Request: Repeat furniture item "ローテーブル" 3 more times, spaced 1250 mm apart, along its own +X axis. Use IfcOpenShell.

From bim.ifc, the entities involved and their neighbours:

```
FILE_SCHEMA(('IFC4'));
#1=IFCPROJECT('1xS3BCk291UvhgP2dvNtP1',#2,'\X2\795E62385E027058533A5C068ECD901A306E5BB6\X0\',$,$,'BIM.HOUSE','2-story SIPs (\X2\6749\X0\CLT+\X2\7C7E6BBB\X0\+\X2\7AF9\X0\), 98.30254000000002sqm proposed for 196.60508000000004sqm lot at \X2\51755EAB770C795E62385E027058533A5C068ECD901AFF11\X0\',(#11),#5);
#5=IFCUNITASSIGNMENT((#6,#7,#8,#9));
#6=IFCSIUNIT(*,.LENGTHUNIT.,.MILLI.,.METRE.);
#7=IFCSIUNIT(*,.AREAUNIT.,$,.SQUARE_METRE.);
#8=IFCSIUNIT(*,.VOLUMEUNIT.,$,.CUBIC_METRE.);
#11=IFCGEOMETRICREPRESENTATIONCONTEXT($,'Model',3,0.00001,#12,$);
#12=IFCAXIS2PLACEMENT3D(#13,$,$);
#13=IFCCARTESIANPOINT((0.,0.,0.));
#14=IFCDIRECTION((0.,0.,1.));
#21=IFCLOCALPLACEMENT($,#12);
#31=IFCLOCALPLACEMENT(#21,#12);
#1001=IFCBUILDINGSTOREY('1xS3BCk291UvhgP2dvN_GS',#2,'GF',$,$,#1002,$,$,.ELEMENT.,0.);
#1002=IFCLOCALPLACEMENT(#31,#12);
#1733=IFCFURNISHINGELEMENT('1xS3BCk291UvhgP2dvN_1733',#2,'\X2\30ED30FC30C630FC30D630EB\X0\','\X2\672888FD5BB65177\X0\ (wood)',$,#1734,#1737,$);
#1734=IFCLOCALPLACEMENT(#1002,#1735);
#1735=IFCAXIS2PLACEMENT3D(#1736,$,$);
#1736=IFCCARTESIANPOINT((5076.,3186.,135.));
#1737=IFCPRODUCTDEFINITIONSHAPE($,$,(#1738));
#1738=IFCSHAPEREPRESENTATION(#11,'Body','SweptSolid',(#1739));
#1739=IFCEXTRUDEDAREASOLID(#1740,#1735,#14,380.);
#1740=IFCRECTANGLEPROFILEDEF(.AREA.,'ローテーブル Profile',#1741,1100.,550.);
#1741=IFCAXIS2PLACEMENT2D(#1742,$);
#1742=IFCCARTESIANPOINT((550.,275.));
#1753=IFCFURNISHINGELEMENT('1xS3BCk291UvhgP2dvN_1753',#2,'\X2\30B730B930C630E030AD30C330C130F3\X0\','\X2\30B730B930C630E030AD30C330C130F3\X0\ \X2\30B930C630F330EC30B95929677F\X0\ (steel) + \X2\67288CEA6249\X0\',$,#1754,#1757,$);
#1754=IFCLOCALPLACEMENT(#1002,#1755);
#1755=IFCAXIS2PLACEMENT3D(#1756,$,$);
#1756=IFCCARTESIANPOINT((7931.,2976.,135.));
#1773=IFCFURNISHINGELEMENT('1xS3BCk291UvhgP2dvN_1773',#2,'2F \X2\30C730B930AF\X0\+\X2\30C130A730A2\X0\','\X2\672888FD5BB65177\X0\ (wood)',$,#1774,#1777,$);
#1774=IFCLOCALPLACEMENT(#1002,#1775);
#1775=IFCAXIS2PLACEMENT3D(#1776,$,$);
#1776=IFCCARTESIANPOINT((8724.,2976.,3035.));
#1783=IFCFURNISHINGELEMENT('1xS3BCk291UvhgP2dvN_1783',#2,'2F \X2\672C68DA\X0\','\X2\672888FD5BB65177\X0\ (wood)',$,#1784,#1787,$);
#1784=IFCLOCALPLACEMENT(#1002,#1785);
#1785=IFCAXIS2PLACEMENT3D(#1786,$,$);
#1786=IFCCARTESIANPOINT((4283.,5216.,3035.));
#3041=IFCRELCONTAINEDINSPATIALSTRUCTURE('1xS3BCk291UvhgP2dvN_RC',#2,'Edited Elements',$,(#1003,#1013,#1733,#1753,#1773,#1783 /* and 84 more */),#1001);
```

```python
import ifcopenshell
import ifcopenshell.api.geometry
import ifcopenshell.api.root
import ifcopenshell.util.element
import ifcopenshell.util.placement
import ifcopenshell.util.unit

model = ifcopenshell.open("bim.ifc")
unit_scale = ifcopenshell.util.unit.calculate_unit_scale(model)


def reuse_history(source, copy):
    """copy_class also copies each property set's owner history, people and application; keep the originals."""
    for rel in copy.IsDefinedBy:
        if rel.is_a("IfcRelDefinesByProperties") and (history := rel.RelatingPropertyDefinition.OwnerHistory):
            rel.RelatingPropertyDefinition.OwnerHistory = source.OwnerHistory
            ifcopenshell.util.element.remove_deep2(model, history)


source = model.by_guid("1xS3BCk291UvhgP2dvN_1733")
base = ifcopenshell.util.placement.get_local_placement(source.ObjectPlacement)
step = base[:3, 0] * 1.25 / unit_scale

for i in range(1, 4):
    copy = ifcopenshell.api.root.copy_class(model, product=source)
    copy.Representation = ifcopenshell.util.element.copy_deep(
        model, source.Representation, exclude=["IfcGeometricRepresentationContext", "IfcRepresentationMap"]
    )
    reuse_history(source, copy)
    matrix = base.copy()
    matrix[:3, 3] += i * step
    print("added at", matrix[:3, 3].round(3) + 0.0)
    ifcopenshell.api.geometry.edit_object_placement(model, product=copy, matrix=matrix, is_si=False)

model.write("bim_updated.ifc")
```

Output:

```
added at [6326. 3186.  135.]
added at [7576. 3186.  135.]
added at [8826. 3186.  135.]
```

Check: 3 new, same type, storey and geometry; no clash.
